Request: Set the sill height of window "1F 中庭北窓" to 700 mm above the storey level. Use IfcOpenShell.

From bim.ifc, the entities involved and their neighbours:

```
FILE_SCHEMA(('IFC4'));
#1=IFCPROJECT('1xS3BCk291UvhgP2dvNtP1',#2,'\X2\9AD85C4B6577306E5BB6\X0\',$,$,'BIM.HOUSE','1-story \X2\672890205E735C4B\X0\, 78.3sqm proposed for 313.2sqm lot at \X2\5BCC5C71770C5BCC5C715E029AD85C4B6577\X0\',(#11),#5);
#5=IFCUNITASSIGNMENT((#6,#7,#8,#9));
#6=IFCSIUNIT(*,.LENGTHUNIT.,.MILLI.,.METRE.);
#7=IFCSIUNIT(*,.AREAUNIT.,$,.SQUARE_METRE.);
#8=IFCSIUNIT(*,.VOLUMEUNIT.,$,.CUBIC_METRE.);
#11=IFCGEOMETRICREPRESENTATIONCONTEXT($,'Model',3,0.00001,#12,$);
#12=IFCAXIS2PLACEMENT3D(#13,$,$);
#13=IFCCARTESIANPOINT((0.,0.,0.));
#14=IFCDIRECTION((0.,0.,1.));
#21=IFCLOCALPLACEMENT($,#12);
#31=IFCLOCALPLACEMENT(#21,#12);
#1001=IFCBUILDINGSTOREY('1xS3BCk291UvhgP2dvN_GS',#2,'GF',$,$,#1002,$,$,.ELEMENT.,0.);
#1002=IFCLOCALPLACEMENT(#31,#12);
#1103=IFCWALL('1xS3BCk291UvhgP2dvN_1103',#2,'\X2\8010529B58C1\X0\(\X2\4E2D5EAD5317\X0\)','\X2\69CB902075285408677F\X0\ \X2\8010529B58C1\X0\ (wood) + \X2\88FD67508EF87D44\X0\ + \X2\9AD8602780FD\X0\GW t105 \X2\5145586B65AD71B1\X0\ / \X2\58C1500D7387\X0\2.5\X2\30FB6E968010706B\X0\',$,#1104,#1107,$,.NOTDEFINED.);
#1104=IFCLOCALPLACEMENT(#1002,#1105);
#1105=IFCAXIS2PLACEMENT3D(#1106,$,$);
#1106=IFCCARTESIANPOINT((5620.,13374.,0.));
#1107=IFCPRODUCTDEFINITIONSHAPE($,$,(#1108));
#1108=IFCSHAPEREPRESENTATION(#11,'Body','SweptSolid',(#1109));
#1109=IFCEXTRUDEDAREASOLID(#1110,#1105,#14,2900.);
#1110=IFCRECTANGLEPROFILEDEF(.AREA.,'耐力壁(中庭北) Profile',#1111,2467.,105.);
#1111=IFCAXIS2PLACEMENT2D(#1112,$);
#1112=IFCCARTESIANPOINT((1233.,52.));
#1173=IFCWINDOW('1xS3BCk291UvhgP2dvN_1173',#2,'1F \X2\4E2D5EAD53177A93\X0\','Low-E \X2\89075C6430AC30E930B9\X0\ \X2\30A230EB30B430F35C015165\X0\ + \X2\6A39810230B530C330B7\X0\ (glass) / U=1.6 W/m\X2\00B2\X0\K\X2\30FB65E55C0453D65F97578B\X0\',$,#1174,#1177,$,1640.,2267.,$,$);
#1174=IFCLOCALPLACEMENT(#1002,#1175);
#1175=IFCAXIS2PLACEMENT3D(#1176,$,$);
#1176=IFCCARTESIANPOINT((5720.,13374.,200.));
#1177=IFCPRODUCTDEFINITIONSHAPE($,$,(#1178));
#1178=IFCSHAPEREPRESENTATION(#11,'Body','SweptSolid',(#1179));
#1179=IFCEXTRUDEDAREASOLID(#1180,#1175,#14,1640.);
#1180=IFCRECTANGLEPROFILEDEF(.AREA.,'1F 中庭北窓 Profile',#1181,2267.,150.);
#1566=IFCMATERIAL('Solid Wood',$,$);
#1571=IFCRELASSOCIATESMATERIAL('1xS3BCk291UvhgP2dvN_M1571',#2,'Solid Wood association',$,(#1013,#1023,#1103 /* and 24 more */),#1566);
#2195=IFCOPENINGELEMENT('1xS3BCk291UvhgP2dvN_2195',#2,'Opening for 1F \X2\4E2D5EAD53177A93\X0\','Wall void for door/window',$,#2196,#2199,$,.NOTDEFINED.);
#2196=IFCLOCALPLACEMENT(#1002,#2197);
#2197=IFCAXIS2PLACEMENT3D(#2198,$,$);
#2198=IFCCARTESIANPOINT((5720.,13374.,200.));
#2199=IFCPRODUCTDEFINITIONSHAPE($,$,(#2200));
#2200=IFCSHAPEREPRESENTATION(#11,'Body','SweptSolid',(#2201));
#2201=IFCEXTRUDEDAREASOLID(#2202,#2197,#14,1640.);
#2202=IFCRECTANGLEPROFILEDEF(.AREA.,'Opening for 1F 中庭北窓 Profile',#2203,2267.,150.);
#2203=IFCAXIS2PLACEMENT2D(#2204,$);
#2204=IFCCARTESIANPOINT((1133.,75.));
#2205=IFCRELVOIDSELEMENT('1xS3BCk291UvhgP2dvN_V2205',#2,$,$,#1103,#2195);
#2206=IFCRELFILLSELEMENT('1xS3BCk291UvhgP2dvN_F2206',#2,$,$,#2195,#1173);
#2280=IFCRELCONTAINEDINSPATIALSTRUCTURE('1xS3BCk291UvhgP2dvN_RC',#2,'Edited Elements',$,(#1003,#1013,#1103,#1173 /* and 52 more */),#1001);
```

```python
import numpy as np
import ifcopenshell
import ifcopenshell.api.geometry
import ifcopenshell.geom
import ifcopenshell.util.element
import ifcopenshell.util.placement
import ifcopenshell.util.shape
import ifcopenshell.util.unit

model = ifcopenshell.open("bim.ifc")
unit_scale = ifcopenshell.util.unit.calculate_unit_scale(model)

window = model.by_guid("1xS3BCk291UvhgP2dvN_1173")
opening = window.FillsVoids[0].RelatingOpeningElement
storey = ifcopenshell.util.element.get_container(window, ifc_class="IfcBuildingStorey")
level = ifcopenshell.util.placement.get_local_placement(storey.ObjectPlacement)[2, 3]

# The opening's origin need not be at the sill, so measure its lowest point.
shape = ifcopenshell.geom.create_shape(ifcopenshell.geom.settings(), opening)
bottom = ifcopenshell.util.shape.get_shape_bottom_elevation(shape, shape.geometry) / unit_scale
dz = level + 700.0 - bottom

shift = np.array([0.0, 0.0, dz])
# The window is not placed relative to its opening, so move both.
for product in (opening, window):
    matrix = ifcopenshell.util.placement.get_local_placement(product.ObjectPlacement)
    matrix[:3, 3] += shift
    ifcopenshell.api.geometry.edit_object_placement(model, product=product, matrix=matrix, is_si=False)

print(f"moved by {dz * unit_scale:+.3f} m")

model.write("bim_edited.ifc")
```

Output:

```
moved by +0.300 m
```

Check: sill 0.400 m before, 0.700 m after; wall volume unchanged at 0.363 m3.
